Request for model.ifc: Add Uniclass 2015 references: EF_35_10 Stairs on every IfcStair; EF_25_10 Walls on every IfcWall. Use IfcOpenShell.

First a look at what the model holds.

```python
import ifcopenshell

model = ifcopenshell.open("model.ifc")
print(model.schema)
print("classifications:", [c.Name for c in model.by_type("IfcClassification")])
for ifc_class in ("IfcDoor", "IfcRoof", "IfcStair", "IfcWall", "IfcWindow"):
    print(ifc_class, len(model.by_type(ifc_class)))
```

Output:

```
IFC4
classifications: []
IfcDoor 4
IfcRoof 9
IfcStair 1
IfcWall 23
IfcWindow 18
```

```python
import ifcopenshell
import ifcopenshell.api.classification

model = ifcopenshell.open("model.ifc")

system = ifcopenshell.api.classification.add_classification(model, classification="Uniclass 2015")

codes = {
    "IfcStair": ("EF_35_10", "Stairs"),
    "IfcWall": ("EF_25_10", "Walls"),
}
for ifc_class, (code, name) in codes.items():
    products = model.by_type(ifc_class)
    ifcopenshell.api.classification.add_reference(
        model, products=products, classification=system, identification=code, name=name
    )
    print(code, len(products))

model.write("model_updated.ifc")
```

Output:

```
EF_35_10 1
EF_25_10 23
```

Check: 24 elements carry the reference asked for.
